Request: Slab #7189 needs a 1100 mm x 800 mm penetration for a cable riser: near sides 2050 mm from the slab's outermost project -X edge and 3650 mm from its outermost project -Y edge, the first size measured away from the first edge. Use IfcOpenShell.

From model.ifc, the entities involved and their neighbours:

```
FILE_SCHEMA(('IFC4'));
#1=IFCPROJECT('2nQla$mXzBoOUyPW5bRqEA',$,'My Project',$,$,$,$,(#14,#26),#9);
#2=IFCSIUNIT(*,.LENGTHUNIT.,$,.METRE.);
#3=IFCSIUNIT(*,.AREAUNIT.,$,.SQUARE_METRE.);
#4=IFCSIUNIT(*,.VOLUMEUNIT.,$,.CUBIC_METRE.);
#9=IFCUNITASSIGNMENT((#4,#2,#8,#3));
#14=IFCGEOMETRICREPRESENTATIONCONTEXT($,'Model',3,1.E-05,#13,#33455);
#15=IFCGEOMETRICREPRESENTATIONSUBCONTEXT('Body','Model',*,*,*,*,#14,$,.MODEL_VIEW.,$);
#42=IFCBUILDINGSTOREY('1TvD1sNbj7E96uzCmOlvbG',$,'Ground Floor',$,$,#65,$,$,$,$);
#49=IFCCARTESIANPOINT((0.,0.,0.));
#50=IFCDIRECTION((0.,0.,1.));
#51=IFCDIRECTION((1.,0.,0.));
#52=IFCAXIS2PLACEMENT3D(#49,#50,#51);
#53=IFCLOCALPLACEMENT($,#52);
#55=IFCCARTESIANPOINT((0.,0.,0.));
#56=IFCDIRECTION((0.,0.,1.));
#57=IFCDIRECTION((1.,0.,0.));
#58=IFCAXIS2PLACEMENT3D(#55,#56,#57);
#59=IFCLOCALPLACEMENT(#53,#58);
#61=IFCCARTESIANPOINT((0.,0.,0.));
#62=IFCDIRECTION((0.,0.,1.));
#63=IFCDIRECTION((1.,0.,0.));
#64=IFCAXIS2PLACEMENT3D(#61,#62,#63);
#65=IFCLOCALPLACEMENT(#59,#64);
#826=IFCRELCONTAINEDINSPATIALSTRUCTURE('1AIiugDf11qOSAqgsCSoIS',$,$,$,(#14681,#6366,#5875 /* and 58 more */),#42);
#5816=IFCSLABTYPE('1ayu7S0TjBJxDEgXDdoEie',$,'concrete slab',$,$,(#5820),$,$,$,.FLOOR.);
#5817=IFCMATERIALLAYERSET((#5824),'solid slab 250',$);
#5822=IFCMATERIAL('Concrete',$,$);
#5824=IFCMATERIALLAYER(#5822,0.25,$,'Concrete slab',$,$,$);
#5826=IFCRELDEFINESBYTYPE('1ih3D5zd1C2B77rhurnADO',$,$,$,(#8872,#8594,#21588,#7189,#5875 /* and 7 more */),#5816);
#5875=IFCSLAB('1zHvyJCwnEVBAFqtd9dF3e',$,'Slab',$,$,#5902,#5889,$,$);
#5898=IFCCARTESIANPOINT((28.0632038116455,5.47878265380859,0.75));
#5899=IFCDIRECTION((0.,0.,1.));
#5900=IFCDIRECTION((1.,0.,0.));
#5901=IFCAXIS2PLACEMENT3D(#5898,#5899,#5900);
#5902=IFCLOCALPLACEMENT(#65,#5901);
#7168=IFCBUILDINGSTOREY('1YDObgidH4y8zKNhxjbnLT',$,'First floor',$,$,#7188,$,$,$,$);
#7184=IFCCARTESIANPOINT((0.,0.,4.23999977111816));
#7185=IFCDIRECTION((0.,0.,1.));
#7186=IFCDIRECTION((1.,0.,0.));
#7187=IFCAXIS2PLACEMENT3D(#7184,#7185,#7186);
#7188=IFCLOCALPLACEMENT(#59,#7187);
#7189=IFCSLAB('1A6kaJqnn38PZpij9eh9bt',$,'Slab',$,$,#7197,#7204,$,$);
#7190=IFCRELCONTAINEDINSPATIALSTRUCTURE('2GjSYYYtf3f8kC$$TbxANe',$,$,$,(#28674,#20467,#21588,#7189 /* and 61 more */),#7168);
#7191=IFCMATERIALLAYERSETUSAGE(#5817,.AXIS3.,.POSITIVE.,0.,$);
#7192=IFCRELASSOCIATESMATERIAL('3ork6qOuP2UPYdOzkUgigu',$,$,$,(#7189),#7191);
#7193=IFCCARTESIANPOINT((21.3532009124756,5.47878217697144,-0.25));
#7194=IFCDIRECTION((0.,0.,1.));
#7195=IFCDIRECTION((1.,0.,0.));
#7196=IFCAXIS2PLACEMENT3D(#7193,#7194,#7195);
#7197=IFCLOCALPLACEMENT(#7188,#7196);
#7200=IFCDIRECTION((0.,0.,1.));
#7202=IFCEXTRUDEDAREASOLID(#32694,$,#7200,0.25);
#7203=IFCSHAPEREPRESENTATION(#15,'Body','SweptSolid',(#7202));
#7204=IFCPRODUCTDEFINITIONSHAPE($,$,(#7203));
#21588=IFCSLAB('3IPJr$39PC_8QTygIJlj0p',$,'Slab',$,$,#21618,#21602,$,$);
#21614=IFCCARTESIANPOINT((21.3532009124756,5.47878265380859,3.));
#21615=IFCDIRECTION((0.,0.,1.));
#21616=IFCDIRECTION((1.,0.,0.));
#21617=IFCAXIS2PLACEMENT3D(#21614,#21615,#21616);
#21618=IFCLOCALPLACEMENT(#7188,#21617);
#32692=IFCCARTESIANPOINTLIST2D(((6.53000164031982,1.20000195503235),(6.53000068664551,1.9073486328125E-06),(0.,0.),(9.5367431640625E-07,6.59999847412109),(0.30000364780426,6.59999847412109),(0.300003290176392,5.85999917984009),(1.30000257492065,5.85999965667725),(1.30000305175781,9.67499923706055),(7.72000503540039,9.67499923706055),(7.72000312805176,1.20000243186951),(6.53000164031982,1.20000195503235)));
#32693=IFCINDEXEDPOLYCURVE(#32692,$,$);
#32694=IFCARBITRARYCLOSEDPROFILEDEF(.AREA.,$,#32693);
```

```python
import numpy as np
import ifcopenshell
import ifcopenshell.api.feature
import ifcopenshell.api.geometry
import ifcopenshell.api.root
import ifcopenshell.geom
import ifcopenshell.util.placement
import ifcopenshell.util.representation
import ifcopenshell.util.shape
import ifcopenshell.util.unit

model = ifcopenshell.open("model.ifc")
unit_scale = ifcopenshell.util.unit.calculate_unit_scale(model)
settings = ifcopenshell.geom.settings()


def volume(element):
    """Net volume in cubic metres, openings subtracted."""
    shape = ifcopenshell.geom.create_shape(settings, element)
    return ifcopenshell.util.shape.get_volume(shape.geometry)


slab = model.by_guid("1A6kaJqnn38PZpij9eh9bt")
before = volume(slab)

# Extent in the slab's own axes, in metres. The edges named are its -X and -Y sides.
slab_shape = ifcopenshell.geom.create_shape(settings, slab)
vertices = ifcopenshell.util.shape.get_vertices(slab_shape.geometry)
x_min, y_min, bottom = vertices.min(axis=0)
top = vertices[:, 2].max()

opening = ifcopenshell.api.root.create_entity(model, ifc_class="IfcOpeningElement", name="Cable riser opening", predefined_type="OPENING")
context = ifcopenshell.util.representation.get_context(model, "Model", "Body", "MODEL_VIEW")
width, depth = 1.1, 0.8
outline = [(0.0, 0.0), (width, 0.0), (width, depth), (0.0, depth), (0.0, 0.0)]
# Overshoot both faces by 50 mm so the cut is clean.
shape = ifcopenshell.api.geometry.add_slab_representation(
    model, context=context, depth=top - bottom + 0.1, polyline=outline
)
ifcopenshell.api.geometry.assign_representation(model, product=opening, representation=shape)

matrix = ifcopenshell.util.placement.get_local_placement(slab.ObjectPlacement)
matrix[:, 3] = matrix @ np.append(np.array([x_min + 2.05, y_min + 3.65, bottom - 0.05]) / unit_scale, 1.0)
ifcopenshell.api.geometry.edit_object_placement(model, product=opening, matrix=matrix, is_si=False)
ifcopenshell.api.feature.add_feature(model, feature=opening, element=slab)

after = volume(slab)

print(f"slab volume {before:.3f} -> {after:.3f} m3")

model.write("model_updated.ifc")
```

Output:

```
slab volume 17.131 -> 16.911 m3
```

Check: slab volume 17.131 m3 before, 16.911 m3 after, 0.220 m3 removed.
